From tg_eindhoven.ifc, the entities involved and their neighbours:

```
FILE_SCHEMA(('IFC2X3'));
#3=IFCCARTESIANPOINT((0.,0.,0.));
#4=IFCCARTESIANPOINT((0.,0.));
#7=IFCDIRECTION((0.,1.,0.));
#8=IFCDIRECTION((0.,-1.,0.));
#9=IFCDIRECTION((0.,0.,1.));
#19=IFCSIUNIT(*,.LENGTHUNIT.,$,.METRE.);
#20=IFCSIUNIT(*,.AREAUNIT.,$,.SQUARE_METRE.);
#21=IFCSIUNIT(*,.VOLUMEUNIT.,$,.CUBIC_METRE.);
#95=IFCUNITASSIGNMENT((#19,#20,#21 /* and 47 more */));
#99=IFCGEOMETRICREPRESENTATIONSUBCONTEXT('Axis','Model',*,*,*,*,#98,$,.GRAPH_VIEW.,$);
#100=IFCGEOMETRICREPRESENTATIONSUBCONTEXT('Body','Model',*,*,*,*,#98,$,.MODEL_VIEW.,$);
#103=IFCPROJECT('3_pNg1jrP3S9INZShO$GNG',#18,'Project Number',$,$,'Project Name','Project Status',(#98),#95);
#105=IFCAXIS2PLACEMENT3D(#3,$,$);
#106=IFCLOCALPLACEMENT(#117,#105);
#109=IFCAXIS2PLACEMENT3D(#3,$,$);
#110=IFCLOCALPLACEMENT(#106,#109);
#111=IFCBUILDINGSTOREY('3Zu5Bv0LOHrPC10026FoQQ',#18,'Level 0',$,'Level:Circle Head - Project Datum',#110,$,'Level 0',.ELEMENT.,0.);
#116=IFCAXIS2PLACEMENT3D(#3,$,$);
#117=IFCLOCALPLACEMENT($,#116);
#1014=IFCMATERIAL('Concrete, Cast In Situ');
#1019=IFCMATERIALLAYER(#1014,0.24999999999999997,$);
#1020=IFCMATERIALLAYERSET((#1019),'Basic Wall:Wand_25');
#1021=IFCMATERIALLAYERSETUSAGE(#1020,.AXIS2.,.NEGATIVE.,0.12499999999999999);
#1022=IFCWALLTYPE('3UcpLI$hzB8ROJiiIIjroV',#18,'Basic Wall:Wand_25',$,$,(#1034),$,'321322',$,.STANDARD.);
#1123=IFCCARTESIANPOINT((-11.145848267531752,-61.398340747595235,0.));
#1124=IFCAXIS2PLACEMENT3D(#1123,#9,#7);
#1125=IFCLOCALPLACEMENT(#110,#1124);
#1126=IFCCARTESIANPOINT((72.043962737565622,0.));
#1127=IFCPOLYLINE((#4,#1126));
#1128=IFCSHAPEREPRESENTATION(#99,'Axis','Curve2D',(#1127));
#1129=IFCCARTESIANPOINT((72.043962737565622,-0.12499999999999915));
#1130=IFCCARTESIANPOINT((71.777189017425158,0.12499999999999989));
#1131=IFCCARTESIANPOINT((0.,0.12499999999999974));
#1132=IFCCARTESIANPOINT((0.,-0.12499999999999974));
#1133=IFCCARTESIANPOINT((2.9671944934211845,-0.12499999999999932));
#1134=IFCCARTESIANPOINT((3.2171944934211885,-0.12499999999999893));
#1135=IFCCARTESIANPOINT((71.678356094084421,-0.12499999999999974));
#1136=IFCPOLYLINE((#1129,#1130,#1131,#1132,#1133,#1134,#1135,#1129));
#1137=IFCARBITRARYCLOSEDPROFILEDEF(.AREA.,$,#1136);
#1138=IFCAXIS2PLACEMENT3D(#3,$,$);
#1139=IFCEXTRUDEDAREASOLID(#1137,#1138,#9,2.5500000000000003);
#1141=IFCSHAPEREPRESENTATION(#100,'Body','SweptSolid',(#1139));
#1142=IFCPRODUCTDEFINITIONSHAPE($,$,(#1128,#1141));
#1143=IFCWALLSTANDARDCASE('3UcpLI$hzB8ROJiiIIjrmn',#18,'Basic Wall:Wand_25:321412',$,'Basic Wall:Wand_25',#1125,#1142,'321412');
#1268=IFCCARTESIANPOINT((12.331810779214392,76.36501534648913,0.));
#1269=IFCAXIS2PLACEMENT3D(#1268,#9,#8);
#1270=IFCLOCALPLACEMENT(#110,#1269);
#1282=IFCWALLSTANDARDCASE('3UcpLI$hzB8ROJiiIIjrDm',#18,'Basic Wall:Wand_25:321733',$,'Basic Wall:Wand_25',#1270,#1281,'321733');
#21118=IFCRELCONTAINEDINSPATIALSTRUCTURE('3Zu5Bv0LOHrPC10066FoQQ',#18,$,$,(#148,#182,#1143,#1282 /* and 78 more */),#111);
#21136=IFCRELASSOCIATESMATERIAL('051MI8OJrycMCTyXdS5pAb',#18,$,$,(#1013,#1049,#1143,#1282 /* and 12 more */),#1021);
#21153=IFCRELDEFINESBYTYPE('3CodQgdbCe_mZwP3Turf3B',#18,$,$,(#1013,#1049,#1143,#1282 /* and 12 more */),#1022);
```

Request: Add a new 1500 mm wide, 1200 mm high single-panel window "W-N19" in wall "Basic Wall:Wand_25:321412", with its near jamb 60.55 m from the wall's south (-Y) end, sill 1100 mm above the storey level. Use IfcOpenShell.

```python
import numpy as np
import ifcopenshell
import ifcopenshell.api.feature
import ifcopenshell.api.geometry
import ifcopenshell.api.root
import ifcopenshell.api.spatial
import ifcopenshell.api.type
import ifcopenshell.geom
import ifcopenshell.util.element
import ifcopenshell.util.placement
import ifcopenshell.util.representation
import ifcopenshell.util.shape
import ifcopenshell.util.unit

model = ifcopenshell.open("tg_eindhoven.ifc")
unit_scale = ifcopenshell.util.unit.calculate_unit_scale(model)
settings = ifcopenshell.geom.settings()


def volume(element):
    """Net volume in cubic metres, openings subtracted."""
    shape = ifcopenshell.geom.create_shape(settings, element)
    return ifcopenshell.util.shape.get_volume(shape.geometry)


wall = model.by_guid("3UcpLI$hzB8ROJiiIIjrmn")
storey = ifcopenshell.util.element.get_container(wall, ifc_class="IfcBuildingStorey")
context = ifcopenshell.util.representation.get_context(model, "Model", "Body", "MODEL_VIEW")
before = volume(wall)

width, height, from_end, sill = 1.5, 1.2, 60.55, 1.1  # metres

# The wall runs along its own X axis, and the end named is its -X end.
wall_shape = ifcopenshell.geom.create_shape(settings, wall)
x, y, z = ifcopenshell.util.shape.get_vertices(wall_shape.geometry).T
start = x.min() + from_end
face, thickness = float(y.min()), float(y.max() - y.min())
wall_matrix = ifcopenshell.util.placement.get_local_placement(wall.ObjectPlacement)
level = ifcopenshell.util.placement.get_local_placement(storey.ObjectPlacement)[2, 3]


def in_wall(x, y):
    """Placement at x, y metres in the wall's axes, at sill height."""
    matrix = wall_matrix.copy()
    matrix[:, 3] = wall_matrix @ np.array([x / unit_scale, y / unit_scale, 0.0, 1.0])
    matrix[2, 3] = level + sill / unit_scale
    return matrix


# Opening: a box that overshoots both wall faces by 50 mm.
opening = ifcopenshell.api.root.create_entity(model, ifc_class="IfcOpeningElement")
box = ifcopenshell.api.geometry.add_wall_representation(
    model, context=context, length=width, height=height, thickness=thickness + 0.1
)
ifcopenshell.api.geometry.assign_representation(model, product=opening, representation=box)
ifcopenshell.api.geometry.edit_object_placement(model, product=opening, matrix=in_wall(start, face - 0.05), is_si=False)
ifcopenshell.api.feature.add_feature(model, feature=opening, element=wall)

window = ifcopenshell.api.root.create_entity(model, ifc_class="IfcWindow", name="W-N19")
window.OverallWidth, window.OverallHeight = width / unit_scale, height / unit_scale
body = ifcopenshell.api.geometry.add_window_representation(
    model,
    context=context,
    overall_width=window.OverallWidth,
    overall_height=window.OverallHeight,
    partition_type="SINGLE_PANEL",
)
ifcopenshell.api.geometry.assign_representation(model, product=window, representation=body)
ifcopenshell.api.spatial.assign_container(model, products=[window], relating_structure=storey)
fills = ifcopenshell.api.feature.add_filling(model, opening=opening, element=window)
fills.OwnerHistory = window.OwnerHistory  # required in IFC2X3

# IFC2X3 keeps the operation on the window style.
style = ifcopenshell.api.root.create_entity(model, ifc_class="IfcWindowStyle", name="W-N19")
style.OperationType, style.ConstructionType = "SINGLE_PANEL", "NOTDEFINED"
style.ParameterTakesPrecedence = style.Sizeable = False
ifcopenshell.api.type.assign_type(model, related_objects=[window], relating_type=style)

# Centre the window in the wall's thickness.
ifcopenshell.api.geometry.edit_object_placement(model, product=window, matrix=in_wall(start, face), is_si=False)
window_shape = ifcopenshell.geom.create_shape(settings, window)
depth = ifcopenshell.util.shape.get_vertices(window_shape.geometry)[:, 1]
offset = face + thickness / 2 - (depth.min() + depth.max()) / 2
ifcopenshell.api.geometry.edit_object_placement(model, product=window, matrix=in_wall(start, offset), is_si=False)

after = volume(wall)

print(f"wall volume {before:.3f} -> {after:.3f} m3")

model.write("tg_eindhoven_updated.ifc")
```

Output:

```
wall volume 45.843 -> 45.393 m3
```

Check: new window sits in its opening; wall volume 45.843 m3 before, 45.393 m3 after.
